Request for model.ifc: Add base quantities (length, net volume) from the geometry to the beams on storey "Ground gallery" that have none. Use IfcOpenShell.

First a look at what the model holds.

```python
import ifcopenshell
import ifcopenshell.util.element
import ifcopenshell.util.unit

model = ifcopenshell.open("model.ifc")
print(model.schema)
for unit_type in ("LENGTHUNIT", "AREAUNIT", "VOLUMEUNIT"):
    print(unit_type, ifcopenshell.util.unit.calculate_unit_scale(model, unit_type))
storey = next(s for s in model.by_type("IfcBuildingStorey") if s.Name == "Ground gallery")
beams = [e for e in ifcopenshell.util.element.get_decomposition(storey) if e.is_a("IfcBeam")]
for e in sorted(beams, key=lambda e: e.id()):
    print(e.id(), e.is_a(), e.Name, list(ifcopenshell.util.element.get_psets(e, qtos_only=True)), sep=" | ")
```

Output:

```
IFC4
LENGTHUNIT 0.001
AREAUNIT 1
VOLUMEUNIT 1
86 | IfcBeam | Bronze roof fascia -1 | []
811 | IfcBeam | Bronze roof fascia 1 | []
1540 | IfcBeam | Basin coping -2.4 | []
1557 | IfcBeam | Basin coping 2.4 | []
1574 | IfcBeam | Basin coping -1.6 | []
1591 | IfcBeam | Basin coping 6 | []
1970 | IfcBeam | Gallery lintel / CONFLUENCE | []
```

```python
import ifcopenshell
import ifcopenshell.api.pset
import ifcopenshell.geom
import ifcopenshell.util.element
import ifcopenshell.util.shape
import ifcopenshell.util.unit

model = ifcopenshell.open("model.ifc")
unit_scale = ifcopenshell.util.unit.calculate_unit_scale(model)
volume_scale = ifcopenshell.util.unit.calculate_unit_scale(model, "VOLUMEUNIT")
settings = ifcopenshell.geom.settings()

storey = next(s for s in model.by_type("IfcBuildingStorey") if s.Name == "Ground gallery")
beams = [e for e in ifcopenshell.util.element.get_decomposition(storey) if e.is_a("IfcBeam")]

for e in sorted(beams, key=lambda e: e.id()):
    if ifcopenshell.util.element.get_psets(e, qtos_only=True, should_inherit=False):
        continue
    # Geometry comes back in metres, in the element's own axes.
    shape = ifcopenshell.geom.create_shape(settings, e)
    values = {
        "Length": ifcopenshell.util.shape.get_max_xyz(shape.geometry) / unit_scale,
        "NetVolume": ifcopenshell.util.shape.get_volume(shape.geometry) / volume_scale,
    }
    qto = ifcopenshell.api.pset.add_qto(model, product=e, name="Qto_BeamBaseQuantities")
    ifcopenshell.api.pset.edit_qto(model, qto=qto, properties=values)
    print(e.id(), {k: round(v, 3) for k, v in values.items()})

model.write("model_v2.ifc")
```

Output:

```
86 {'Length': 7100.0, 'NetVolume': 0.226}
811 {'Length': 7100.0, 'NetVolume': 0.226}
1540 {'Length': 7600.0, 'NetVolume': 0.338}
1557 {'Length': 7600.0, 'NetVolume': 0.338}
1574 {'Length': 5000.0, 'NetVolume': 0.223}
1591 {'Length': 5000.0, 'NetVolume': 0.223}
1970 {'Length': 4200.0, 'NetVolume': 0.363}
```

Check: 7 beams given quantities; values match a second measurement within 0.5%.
